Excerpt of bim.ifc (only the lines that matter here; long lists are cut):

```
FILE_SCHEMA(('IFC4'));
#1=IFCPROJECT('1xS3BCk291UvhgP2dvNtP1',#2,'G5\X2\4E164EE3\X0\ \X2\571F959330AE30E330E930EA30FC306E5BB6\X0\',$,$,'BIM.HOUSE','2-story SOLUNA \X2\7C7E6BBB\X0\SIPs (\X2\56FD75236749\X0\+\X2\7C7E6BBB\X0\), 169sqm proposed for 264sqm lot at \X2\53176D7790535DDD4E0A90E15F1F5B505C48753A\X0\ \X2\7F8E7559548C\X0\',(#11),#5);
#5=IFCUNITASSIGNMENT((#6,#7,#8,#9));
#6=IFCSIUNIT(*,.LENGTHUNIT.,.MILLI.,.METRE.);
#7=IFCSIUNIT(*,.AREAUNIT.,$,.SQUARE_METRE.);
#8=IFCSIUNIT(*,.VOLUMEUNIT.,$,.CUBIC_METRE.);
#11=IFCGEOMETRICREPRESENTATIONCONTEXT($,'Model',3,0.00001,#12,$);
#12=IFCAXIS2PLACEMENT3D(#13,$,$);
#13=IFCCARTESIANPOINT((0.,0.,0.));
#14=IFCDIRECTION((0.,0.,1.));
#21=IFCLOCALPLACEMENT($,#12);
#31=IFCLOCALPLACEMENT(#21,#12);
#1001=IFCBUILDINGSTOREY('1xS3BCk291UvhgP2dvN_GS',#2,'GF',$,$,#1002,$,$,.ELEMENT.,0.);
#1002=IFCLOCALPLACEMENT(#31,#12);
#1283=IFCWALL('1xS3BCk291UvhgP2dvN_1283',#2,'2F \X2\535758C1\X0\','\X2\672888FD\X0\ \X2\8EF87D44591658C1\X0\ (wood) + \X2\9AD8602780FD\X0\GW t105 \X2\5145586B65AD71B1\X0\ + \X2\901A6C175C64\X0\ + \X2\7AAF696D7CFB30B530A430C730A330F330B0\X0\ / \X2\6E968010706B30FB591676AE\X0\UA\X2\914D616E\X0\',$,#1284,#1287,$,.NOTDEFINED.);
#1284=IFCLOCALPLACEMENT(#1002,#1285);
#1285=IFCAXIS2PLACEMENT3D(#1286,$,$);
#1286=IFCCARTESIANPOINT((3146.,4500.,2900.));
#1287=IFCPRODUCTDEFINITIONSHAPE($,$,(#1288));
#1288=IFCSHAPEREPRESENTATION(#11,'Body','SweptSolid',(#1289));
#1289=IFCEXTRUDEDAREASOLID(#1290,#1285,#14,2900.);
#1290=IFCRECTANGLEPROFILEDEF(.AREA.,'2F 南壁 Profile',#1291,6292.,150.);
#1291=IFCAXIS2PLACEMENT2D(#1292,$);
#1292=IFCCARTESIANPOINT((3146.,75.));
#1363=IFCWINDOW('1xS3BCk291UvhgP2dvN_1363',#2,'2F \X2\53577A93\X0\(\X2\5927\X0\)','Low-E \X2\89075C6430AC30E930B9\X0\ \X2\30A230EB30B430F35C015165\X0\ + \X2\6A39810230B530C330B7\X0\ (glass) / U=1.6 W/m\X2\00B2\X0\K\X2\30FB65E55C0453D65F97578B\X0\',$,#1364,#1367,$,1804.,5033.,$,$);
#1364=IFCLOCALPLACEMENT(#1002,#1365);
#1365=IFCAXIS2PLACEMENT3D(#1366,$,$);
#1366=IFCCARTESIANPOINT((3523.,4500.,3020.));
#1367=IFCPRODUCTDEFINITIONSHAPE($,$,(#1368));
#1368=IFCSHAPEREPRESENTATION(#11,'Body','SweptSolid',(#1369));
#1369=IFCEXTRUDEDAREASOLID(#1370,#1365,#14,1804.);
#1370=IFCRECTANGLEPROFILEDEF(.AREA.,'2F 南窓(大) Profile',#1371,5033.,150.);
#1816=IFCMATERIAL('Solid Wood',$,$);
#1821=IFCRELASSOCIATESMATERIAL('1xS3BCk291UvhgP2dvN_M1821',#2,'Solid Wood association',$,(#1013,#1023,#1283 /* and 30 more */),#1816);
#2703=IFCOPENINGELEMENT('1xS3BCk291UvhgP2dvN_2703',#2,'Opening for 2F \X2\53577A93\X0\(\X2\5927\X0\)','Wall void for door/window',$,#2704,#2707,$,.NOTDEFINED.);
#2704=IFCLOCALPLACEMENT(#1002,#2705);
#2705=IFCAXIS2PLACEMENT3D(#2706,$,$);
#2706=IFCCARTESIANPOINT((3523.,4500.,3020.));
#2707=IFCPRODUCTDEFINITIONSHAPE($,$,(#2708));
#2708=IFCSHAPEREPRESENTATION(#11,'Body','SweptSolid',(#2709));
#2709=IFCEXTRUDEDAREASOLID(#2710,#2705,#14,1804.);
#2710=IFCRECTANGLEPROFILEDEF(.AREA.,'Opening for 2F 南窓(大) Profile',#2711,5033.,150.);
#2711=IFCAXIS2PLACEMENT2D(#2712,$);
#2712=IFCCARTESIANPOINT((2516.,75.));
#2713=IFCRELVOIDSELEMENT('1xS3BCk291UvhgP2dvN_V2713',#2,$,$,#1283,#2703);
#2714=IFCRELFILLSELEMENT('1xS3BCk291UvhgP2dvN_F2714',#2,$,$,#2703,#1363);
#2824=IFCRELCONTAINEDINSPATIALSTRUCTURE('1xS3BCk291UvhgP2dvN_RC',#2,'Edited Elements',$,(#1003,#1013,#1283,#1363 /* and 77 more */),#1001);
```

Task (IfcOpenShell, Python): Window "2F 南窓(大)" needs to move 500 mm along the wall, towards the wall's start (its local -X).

```python
import ifcopenshell
import ifcopenshell.api.geometry
import ifcopenshell.util.placement
import ifcopenshell.util.unit

model = ifcopenshell.open("bim.ifc")
unit_scale = ifcopenshell.util.unit.calculate_unit_scale(model)

window = model.by_guid("1xS3BCk291UvhgP2dvN_1363")
opening = window.FillsVoids[0].RelatingOpeningElement
wall = opening.VoidsElements[0].RelatingBuildingElement

wall_matrix = ifcopenshell.util.placement.get_local_placement(wall.ObjectPlacement)
shift = wall_matrix[:3, 0] * -0.5 / unit_scale
before = ifcopenshell.util.placement.get_local_placement(window.ObjectPlacement)[:3, 3].copy()

# The window is not placed relative to its opening, so move both.
for product in (opening, window):
    matrix = ifcopenshell.util.placement.get_local_placement(product.ObjectPlacement)
    matrix[:3, 3] += shift
    ifcopenshell.api.geometry.edit_object_placement(model, product=product, matrix=matrix, is_si=False)

after = ifcopenshell.util.placement.get_local_placement(window.ObjectPlacement)[:3, 3]
print("window moved by", (after - before).round(3) + 0.0)

model.write("bim_v2.ifc")
```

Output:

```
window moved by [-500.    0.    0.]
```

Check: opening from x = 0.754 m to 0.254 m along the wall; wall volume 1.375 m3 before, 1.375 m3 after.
